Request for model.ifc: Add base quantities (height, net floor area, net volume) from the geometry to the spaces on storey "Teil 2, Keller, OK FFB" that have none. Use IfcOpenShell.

First a look at what the model holds.

```python
import ifcopenshell
import ifcopenshell.util.element
import ifcopenshell.util.unit

model = ifcopenshell.open("model.ifc")
print(model.schema)
for unit_type in ("LENGTHUNIT", "AREAUNIT", "VOLUMEUNIT"):
    print(unit_type, ifcopenshell.util.unit.calculate_unit_scale(model, unit_type))
storey = next(s for s in model.by_type("IfcBuildingStorey") if s.Name == "Teil 2, Keller, OK FFB")
spaces = [e for e in ifcopenshell.util.element.get_decomposition(storey) if e.is_a("IfcSpace")]
for e in sorted(spaces, key=lambda e: e.id()):
    print(e.id(), e.is_a(), e.Name, list(ifcopenshell.util.element.get_psets(e, qtos_only=True)), sep=" | ")
```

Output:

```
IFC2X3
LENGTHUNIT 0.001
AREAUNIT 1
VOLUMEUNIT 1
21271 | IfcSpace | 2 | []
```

```python
import ifcopenshell
import ifcopenshell.api.pset
import ifcopenshell.geom
import ifcopenshell.util.element
import ifcopenshell.util.shape
import ifcopenshell.util.unit

model = ifcopenshell.open("model.ifc")
unit_scale = ifcopenshell.util.unit.calculate_unit_scale(model)
area_scale = ifcopenshell.util.unit.calculate_unit_scale(model, "AREAUNIT")
volume_scale = ifcopenshell.util.unit.calculate_unit_scale(model, "VOLUMEUNIT")
settings = ifcopenshell.geom.settings()

storey = next(s for s in model.by_type("IfcBuildingStorey") if s.Name == "Teil 2, Keller, OK FFB")
spaces = [e for e in ifcopenshell.util.element.get_decomposition(storey) if e.is_a("IfcSpace")]

for e in sorted(spaces, key=lambda e: e.id()):
    if ifcopenshell.util.element.get_psets(e, qtos_only=True, should_inherit=False):
        continue
    # Geometry comes back in metres, in the element's own axes.
    shape = ifcopenshell.geom.create_shape(settings, e)
    values = {
        "Height": ifcopenshell.util.shape.get_z(shape.geometry) / unit_scale,
        "NetFloorArea": ifcopenshell.util.shape.get_footprint_area(shape.geometry) / area_scale,
        "NetVolume": ifcopenshell.util.shape.get_volume(shape.geometry) / volume_scale,
    }
    qto = ifcopenshell.api.pset.add_qto(model, product=e, name="BaseQuantities")
    ifcopenshell.api.pset.edit_qto(model, qto=qto, properties=values)
    print(e.id(), {k: round(v, 3) for k, v in values.items()})

model.write("model_rev.ifc")
```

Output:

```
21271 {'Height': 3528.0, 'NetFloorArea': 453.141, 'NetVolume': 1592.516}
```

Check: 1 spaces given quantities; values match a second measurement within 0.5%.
